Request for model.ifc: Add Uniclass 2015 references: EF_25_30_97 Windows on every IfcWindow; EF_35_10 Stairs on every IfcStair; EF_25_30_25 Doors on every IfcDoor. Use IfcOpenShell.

First a look at what the model holds.

```python
import ifcopenshell

model = ifcopenshell.open("model.ifc")
print(model.schema)
print("classifications:", [c.Name for c in model.by_type("IfcClassification")])
for ifc_class in ("IfcDoor", "IfcRoof", "IfcStair", "IfcWall", "IfcWindow"):
    print(ifc_class, len(model.by_type(ifc_class)))
```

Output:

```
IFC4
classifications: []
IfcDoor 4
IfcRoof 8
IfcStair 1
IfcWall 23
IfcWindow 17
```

```python
import ifcopenshell
import ifcopenshell.api.classification

model = ifcopenshell.open("model.ifc")

system = ifcopenshell.api.classification.add_classification(model, classification="Uniclass 2015")

codes = {
    "IfcWindow": ("EF_25_30_97", "Windows"),
    "IfcStair": ("EF_35_10", "Stairs"),
    "IfcDoor": ("EF_25_30_25", "Doors"),
}
for ifc_class, (code, name) in codes.items():
    products = model.by_type(ifc_class)
    ifcopenshell.api.classification.add_reference(
        model, products=products, classification=system, identification=code, name=name
    )
    print(code, len(products))

model.write("model_updated.ifc")
```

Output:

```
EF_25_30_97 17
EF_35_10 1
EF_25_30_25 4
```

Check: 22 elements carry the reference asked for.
